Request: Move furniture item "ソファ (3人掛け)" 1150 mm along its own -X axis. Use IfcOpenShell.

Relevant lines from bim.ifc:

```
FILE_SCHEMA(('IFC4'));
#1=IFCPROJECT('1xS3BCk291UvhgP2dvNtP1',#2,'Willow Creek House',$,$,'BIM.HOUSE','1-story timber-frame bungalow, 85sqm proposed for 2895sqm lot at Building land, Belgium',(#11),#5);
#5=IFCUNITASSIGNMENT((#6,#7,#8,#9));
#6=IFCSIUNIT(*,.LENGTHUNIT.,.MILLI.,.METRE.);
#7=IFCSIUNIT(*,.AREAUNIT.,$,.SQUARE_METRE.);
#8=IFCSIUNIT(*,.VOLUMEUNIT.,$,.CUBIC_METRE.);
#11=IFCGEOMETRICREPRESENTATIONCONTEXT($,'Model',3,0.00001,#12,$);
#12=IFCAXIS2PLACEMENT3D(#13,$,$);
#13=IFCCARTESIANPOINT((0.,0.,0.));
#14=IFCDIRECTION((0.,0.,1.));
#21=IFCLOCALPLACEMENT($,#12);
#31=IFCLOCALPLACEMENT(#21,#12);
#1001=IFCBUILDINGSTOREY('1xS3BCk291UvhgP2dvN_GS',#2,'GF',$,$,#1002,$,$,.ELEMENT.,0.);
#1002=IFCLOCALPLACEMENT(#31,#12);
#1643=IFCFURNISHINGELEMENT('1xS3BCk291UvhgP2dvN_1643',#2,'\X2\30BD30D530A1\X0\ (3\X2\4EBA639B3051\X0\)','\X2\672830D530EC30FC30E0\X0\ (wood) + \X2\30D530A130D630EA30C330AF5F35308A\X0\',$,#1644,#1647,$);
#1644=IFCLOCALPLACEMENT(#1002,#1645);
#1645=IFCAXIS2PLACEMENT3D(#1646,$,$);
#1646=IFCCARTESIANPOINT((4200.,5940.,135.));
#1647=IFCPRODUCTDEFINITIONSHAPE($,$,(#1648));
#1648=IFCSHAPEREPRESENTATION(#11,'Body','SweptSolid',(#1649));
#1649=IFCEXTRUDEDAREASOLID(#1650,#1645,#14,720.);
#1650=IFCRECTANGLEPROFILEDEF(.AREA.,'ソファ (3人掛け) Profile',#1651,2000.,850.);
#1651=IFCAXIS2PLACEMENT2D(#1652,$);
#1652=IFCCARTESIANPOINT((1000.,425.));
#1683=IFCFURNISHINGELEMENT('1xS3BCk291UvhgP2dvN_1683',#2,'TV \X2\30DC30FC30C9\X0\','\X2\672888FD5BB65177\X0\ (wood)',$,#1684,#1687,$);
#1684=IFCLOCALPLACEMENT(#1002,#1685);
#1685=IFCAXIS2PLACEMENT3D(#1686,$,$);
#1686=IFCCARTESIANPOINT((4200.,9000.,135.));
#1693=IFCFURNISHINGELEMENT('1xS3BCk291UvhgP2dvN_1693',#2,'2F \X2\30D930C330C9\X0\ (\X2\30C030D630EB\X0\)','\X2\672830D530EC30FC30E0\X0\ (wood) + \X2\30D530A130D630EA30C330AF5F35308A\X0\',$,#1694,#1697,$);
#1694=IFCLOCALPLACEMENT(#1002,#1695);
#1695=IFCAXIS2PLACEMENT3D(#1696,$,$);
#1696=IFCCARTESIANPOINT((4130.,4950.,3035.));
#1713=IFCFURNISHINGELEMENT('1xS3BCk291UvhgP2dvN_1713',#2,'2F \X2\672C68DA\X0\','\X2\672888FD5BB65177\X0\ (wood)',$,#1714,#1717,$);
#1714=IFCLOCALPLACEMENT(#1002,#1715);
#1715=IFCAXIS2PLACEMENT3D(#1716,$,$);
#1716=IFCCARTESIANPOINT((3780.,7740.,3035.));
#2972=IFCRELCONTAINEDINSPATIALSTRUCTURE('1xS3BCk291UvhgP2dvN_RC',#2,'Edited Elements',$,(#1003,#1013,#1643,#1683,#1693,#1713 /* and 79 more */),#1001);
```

```python
import ifcopenshell
import ifcopenshell.api.geometry
import ifcopenshell.util.placement

model = ifcopenshell.open("bim.ifc")

item = model.by_guid("1xS3BCk291UvhgP2dvN_1643")
matrix = ifcopenshell.util.placement.get_local_placement(item.ObjectPlacement)
matrix[:3, 3] -= matrix[:3, 0] * 1150.0
ifcopenshell.api.geometry.edit_object_placement(model, product=item, matrix=matrix, is_si=False)

print(ifcopenshell.util.placement.get_local_placement(item.ObjectPlacement).round(3) + 0.0)

model.write("bim_updated.ifc")
```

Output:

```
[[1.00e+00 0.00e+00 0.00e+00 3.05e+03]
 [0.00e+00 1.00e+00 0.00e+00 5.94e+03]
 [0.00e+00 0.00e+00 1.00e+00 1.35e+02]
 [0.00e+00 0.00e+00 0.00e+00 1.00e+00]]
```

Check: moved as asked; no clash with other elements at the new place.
